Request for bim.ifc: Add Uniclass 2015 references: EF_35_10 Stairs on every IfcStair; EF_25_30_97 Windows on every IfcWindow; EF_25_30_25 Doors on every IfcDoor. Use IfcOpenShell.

First a look at what the model holds.

```python
import ifcopenshell

model = ifcopenshell.open("bim.ifc")
print(model.schema)
print("classifications:", [c.Name for c in model.by_type("IfcClassification")])
for ifc_class in ("IfcDoor", "IfcRoof", "IfcStair", "IfcWall", "IfcWindow"):
    print(ifc_class, len(model.by_type(ifc_class)))
```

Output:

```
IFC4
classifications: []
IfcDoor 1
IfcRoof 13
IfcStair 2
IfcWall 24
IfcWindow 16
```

```python
import ifcopenshell
import ifcopenshell.api.classification

model = ifcopenshell.open("bim.ifc")

system = ifcopenshell.api.classification.add_classification(model, classification="Uniclass 2015")

codes = {
    "IfcStair": ("EF_35_10", "Stairs"),
    "IfcWindow": ("EF_25_30_97", "Windows"),
    "IfcDoor": ("EF_25_30_25", "Doors"),
}
for ifc_class, (code, name) in codes.items():
    products = model.by_type(ifc_class)
    ifcopenshell.api.classification.add_reference(
        model, products=products, classification=system, identification=code, name=name
    )
    print(code, len(products))

model.write("bim_edited.ifc")
```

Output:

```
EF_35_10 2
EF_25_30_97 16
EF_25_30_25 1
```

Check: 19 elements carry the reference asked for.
